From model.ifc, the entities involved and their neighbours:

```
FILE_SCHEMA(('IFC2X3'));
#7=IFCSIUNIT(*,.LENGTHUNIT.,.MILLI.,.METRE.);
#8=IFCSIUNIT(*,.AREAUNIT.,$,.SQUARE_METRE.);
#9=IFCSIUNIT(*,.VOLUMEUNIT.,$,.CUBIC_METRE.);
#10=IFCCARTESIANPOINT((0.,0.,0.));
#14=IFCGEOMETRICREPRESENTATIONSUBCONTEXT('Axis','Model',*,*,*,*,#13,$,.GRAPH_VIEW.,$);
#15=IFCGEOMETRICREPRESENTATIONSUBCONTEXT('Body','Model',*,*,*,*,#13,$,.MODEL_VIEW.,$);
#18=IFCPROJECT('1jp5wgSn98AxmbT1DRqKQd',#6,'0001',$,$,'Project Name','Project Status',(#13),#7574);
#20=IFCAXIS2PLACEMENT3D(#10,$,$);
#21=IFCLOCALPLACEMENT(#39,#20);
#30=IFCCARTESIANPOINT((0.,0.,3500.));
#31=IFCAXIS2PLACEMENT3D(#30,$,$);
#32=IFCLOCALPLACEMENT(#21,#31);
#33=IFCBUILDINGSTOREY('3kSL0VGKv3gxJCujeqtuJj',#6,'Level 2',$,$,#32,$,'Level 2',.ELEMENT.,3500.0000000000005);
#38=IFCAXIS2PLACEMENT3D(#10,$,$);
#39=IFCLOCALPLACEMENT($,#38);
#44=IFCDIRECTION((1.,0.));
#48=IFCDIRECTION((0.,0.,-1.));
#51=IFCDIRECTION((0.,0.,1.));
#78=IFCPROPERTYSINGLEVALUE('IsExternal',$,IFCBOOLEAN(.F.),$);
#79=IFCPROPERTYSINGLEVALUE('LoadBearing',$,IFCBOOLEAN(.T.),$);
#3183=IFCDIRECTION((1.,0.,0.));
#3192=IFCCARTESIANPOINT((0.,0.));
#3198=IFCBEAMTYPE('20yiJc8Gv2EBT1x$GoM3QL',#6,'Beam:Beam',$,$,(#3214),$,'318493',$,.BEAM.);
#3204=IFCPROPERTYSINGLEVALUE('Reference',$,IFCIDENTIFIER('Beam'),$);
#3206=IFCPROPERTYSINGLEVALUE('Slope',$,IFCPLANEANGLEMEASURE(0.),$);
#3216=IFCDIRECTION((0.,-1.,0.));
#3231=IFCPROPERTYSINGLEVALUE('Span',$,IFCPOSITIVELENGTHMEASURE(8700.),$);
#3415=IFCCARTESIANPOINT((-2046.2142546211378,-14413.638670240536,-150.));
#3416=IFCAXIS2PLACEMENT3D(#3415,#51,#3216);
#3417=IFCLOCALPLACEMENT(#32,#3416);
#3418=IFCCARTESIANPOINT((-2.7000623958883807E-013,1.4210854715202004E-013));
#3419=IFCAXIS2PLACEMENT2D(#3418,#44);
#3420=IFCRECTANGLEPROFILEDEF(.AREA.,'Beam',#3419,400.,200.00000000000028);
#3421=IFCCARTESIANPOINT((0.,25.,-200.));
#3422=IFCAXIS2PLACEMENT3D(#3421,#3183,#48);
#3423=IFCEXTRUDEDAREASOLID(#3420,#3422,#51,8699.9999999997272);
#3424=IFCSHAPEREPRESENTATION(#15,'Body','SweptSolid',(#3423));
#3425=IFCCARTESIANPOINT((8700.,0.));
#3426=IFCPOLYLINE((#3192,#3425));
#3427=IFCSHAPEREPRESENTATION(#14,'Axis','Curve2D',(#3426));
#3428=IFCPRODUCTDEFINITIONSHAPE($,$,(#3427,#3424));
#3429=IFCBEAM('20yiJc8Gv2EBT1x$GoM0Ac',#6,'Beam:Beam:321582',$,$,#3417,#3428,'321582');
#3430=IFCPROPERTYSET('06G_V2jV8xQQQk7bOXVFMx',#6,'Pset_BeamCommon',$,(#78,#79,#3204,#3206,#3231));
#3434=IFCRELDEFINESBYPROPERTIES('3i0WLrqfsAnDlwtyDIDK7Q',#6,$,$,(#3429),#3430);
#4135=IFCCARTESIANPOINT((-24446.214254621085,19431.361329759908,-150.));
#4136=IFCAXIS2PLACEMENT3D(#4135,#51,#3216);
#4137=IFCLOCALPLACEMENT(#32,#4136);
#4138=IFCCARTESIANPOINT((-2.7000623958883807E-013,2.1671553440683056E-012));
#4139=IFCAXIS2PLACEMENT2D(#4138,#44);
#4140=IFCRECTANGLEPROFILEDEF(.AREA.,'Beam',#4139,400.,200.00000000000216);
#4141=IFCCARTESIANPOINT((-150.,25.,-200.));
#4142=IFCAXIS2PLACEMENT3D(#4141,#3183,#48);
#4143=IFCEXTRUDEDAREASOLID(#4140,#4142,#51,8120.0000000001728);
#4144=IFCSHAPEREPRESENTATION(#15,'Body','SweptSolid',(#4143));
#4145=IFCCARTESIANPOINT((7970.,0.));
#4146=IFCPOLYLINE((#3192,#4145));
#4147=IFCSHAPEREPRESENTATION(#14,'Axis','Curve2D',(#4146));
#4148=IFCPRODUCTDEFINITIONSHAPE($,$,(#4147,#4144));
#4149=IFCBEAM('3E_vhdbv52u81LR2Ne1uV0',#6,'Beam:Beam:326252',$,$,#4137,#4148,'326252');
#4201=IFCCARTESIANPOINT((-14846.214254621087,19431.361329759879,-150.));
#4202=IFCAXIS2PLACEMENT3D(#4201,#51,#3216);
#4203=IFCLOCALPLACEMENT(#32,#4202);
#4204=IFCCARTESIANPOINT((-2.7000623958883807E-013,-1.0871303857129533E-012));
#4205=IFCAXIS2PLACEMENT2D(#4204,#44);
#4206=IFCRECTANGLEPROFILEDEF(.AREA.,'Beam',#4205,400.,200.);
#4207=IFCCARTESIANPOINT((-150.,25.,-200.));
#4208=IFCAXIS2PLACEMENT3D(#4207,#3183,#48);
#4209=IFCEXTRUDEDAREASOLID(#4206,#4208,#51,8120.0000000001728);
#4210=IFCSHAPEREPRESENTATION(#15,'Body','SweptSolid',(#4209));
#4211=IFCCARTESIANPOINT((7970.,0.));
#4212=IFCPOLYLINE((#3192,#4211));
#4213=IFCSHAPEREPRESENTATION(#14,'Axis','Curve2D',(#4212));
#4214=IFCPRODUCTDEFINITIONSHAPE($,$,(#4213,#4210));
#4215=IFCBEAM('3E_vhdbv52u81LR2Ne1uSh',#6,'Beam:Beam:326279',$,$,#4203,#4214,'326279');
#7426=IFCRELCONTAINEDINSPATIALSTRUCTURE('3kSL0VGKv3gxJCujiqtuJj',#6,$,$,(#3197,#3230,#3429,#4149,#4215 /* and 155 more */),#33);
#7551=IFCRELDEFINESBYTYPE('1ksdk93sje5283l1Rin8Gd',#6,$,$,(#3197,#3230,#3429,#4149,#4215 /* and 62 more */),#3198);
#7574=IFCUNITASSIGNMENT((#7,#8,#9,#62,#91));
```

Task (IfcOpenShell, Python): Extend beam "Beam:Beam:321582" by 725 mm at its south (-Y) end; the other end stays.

```python
import numpy as np
import ifcopenshell
import ifcopenshell.api.pset
import ifcopenshell.util.element
import ifcopenshell.util.representation
import ifcopenshell.util.unit

model = ifcopenshell.open("model.ifc")
unit_scale = ifcopenshell.util.unit.calculate_unit_scale(model)

member = model.by_guid("20yiJc8Gv2EBT1x$GoM0Ac")
change = 0.725 / unit_scale

# The extrusion runs towards the end named, so only its depth changes.
body = ifcopenshell.util.representation.get_representation(member, "Model", "Body")
solid = body.Items[0]
old_length = solid.Depth
solid.Depth += change

# Move the axis end point with it.
axis = next(r for r in member.Representation.Representations if r.RepresentationIdentifier == "Axis").Items[0]
start, end = (np.array(p.Coordinates) for p in axis.Points)
end = end + (end - start) / np.linalg.norm(end - start) * change
point = model.createIfcCartesianPoint(end.tolist())
axis.Points = [axis.Points[0], point]

# Update the stored length and volume.
pset = model.by_id(ifcopenshell.util.element.get_pset(member, "Pset_BeamCommon", should_inherit=False)["id"])
ifcopenshell.api.pset.edit_pset(model, pset=pset, properties={
    "Span": model.create_entity("IfcPositiveLengthMeasure", solid.Depth),
})

print(f"length {old_length:g} -> {solid.Depth:g}")

model.write("model-out.ifc")
```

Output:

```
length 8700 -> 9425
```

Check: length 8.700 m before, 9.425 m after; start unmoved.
